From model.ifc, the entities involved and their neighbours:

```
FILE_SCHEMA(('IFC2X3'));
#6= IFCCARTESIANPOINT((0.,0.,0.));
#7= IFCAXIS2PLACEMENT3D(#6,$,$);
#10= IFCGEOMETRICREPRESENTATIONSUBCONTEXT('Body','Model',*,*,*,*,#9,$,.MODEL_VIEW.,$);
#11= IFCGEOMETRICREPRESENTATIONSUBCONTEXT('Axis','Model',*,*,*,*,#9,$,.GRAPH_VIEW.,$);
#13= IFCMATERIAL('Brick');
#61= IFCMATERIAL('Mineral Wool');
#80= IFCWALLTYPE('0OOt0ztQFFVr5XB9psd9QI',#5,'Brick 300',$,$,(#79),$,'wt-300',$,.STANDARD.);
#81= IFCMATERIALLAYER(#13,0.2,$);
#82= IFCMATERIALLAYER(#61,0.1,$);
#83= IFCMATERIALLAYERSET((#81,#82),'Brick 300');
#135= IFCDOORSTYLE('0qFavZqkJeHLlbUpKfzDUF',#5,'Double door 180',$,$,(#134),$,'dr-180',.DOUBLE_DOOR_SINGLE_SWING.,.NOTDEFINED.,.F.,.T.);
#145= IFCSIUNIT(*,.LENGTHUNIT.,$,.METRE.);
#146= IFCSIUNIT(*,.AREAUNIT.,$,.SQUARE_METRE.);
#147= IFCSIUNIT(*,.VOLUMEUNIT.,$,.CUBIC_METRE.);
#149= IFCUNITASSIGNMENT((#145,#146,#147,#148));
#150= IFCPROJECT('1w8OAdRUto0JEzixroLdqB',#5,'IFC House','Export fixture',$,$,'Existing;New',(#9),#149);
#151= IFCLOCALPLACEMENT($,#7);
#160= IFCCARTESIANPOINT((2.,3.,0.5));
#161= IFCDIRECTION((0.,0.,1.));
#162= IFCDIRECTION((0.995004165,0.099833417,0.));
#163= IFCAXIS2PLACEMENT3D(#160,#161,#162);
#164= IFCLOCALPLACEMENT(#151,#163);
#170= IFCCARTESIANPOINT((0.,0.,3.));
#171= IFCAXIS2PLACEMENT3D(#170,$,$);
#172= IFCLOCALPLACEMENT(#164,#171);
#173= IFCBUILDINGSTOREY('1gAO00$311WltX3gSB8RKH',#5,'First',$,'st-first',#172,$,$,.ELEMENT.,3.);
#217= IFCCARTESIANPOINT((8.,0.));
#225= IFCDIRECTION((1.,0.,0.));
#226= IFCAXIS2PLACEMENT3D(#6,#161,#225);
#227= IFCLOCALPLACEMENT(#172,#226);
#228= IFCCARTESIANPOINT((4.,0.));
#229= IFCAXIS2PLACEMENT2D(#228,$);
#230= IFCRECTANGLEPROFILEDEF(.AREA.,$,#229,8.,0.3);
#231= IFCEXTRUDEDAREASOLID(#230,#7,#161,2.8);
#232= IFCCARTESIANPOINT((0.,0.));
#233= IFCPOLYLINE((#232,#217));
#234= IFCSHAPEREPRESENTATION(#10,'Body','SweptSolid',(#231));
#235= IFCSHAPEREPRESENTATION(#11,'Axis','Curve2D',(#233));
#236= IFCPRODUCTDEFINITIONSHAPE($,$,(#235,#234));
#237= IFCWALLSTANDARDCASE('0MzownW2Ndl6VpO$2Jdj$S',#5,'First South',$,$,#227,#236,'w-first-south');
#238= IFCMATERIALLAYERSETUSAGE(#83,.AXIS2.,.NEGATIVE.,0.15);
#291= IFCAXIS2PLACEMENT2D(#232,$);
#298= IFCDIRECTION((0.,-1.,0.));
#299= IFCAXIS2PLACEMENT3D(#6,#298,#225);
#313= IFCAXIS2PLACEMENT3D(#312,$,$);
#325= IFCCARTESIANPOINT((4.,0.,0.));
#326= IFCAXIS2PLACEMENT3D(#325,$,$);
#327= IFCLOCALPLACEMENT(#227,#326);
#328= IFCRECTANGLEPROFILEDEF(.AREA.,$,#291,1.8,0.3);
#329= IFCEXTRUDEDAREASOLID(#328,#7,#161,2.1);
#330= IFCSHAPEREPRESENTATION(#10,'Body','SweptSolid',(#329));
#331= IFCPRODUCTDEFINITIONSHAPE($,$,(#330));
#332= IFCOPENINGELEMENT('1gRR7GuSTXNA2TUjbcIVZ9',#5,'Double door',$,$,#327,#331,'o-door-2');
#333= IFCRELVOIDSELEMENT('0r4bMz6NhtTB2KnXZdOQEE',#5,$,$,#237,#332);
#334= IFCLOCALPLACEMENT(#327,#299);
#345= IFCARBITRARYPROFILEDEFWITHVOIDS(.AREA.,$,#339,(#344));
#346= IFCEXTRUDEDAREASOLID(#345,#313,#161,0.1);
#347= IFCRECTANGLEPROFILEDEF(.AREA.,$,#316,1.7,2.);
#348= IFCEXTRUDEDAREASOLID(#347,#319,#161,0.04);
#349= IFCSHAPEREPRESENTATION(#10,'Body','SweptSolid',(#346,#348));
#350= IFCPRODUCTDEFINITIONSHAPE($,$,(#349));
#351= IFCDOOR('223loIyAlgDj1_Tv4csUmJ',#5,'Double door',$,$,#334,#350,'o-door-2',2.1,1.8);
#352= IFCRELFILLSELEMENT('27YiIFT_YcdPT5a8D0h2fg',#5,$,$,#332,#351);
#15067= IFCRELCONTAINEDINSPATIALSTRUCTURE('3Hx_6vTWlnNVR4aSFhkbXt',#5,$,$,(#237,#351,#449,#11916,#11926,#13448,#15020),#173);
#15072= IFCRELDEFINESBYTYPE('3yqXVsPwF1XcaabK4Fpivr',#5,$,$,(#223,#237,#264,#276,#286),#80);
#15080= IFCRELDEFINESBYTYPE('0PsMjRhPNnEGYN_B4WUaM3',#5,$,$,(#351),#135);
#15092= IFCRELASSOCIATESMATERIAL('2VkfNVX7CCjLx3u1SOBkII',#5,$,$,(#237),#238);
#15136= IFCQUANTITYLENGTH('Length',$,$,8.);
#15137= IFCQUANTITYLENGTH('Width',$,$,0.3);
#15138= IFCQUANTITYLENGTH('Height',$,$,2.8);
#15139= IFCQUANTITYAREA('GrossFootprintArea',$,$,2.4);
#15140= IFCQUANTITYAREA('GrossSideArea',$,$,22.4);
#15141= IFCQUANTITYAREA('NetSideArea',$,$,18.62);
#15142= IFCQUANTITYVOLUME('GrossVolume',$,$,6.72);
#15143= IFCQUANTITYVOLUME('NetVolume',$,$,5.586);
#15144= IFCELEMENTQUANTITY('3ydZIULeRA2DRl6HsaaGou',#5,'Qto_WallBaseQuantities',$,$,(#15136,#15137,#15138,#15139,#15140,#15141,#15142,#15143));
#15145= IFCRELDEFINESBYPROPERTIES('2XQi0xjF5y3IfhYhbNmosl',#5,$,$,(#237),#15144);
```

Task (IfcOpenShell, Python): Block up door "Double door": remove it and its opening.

```python
import ifcopenshell
import ifcopenshell.api.feature
import ifcopenshell.api.pset
import ifcopenshell.api.root
import ifcopenshell.geom
import ifcopenshell.util.element
import ifcopenshell.util.shape
import ifcopenshell.util.unit

model = ifcopenshell.open("model.ifc")
area_scale = ifcopenshell.util.unit.calculate_unit_scale(model, "AREAUNIT")
volume_scale = ifcopenshell.util.unit.calculate_unit_scale(model, "VOLUMEUNIT")
settings = ifcopenshell.geom.settings()


def volume(element):
    """Net volume in cubic metres, openings subtracted."""
    shape = ifcopenshell.geom.create_shape(settings, element)
    return ifcopenshell.util.shape.get_volume(shape.geometry)


door = model.by_guid("223loIyAlgDj1_Tv4csUmJ")
opening = door.FillsVoids[0].RelatingOpeningElement
wall = opening.VoidsElements[0].RelatingBuildingElement
before = volume(wall)

ifcopenshell.api.root.remove_product(model, product=door)
ifcopenshell.api.feature.remove_feature(model, feature=opening)

after = volume(wall)
thickness = 0.3  # wall thickness in metres

# Update the wall's stored quantities.
qto = model.by_id(ifcopenshell.util.element.get_pset(wall, "Qto_WallBaseQuantities", should_inherit=False)["id"])
ifcopenshell.api.pset.edit_qto(model, qto=qto, properties={
    "NetSideArea": after / thickness / area_scale,
    "NetVolume": after / volume_scale,
})

print(f"wall volume {before:.3f} -> {after:.3f} m3")

model.write("model_rev.ifc")
```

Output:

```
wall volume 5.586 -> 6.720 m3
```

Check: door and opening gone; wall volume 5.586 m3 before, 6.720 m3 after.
